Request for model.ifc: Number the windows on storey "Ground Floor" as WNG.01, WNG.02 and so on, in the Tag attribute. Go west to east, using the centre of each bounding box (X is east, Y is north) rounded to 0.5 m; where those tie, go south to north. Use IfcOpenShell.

First a look at what the model holds.

```python
import ifcopenshell
import ifcopenshell.util.element
import ifcopenshell.util.placement

model = ifcopenshell.open("model.ifc")
print(model.schema)
storey = next(s for s in model.by_type("IfcBuildingStorey") if s.Name == "Ground Floor")
windows = [e for e in ifcopenshell.util.element.get_decomposition(storey) if e.is_a("IfcWindow")]
for e in sorted(windows, key=lambda e: e.id()):
    origin = ifcopenshell.util.placement.get_local_placement(e.ObjectPlacement)[:3, 3]
    print(e.id(), e.Tag, e.Name, origin.round(2) + 0.0, sep=" | ")
```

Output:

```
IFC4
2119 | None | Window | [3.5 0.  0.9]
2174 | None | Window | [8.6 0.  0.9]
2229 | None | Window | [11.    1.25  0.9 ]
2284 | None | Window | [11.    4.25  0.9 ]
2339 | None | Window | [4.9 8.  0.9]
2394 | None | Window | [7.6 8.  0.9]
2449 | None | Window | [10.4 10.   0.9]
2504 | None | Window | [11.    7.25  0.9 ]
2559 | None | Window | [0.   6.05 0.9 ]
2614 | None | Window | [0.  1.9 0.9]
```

```python
import ifcopenshell
import ifcopenshell.geom
import ifcopenshell.util.element
import ifcopenshell.util.shape

model = ifcopenshell.open("model.ifc")
settings = ifcopenshell.geom.settings()
settings.set("use-world-coords", True)


def centre(element):
    shape = ifcopenshell.geom.create_shape(settings, element)
    return ifcopenshell.util.shape.get_bbox_centroid(shape.geometry)


storey = next(s for s in model.by_type("IfcBuildingStorey") if s.Name == "Ground Floor")
windows = [e for e in ifcopenshell.util.element.get_decomposition(storey) if e.is_a("IfcWindow")]

# Insertion points can sit at a corner or the storey origin, so sort by the geometry (in metres).
centres = {e: centre(e) for e in windows}
windows.sort(key=lambda e: (round(centres[e][0] / 0.5), centres[e][1]))

for i, e in enumerate(windows, start=1):
    number = f"WNG.{i:02d}"
    e.Tag = number
    print(e.id(), number)

model.write("model_edited.ifc")
```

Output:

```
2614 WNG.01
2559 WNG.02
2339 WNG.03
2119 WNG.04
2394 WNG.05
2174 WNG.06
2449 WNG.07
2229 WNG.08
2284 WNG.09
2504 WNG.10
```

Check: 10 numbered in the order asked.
